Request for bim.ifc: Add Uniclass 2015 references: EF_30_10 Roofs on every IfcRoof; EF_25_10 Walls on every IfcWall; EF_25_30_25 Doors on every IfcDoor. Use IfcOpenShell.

First a look at what the model holds.

```python
import ifcopenshell

model = ifcopenshell.open("bim.ifc")
print(model.schema)
print("classifications:", [c.Name for c in model.by_type("IfcClassification")])
for ifc_class in ("IfcDoor", "IfcRoof", "IfcStair", "IfcWall", "IfcWindow"):
    print(ifc_class, len(model.by_type(ifc_class)))
```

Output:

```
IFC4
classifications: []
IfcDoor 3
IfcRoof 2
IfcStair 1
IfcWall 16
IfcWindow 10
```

```python
import ifcopenshell
import ifcopenshell.api.classification

model = ifcopenshell.open("bim.ifc")

system = ifcopenshell.api.classification.add_classification(model, classification="Uniclass 2015")

codes = {
    "IfcRoof": ("EF_30_10", "Roofs"),
    "IfcWall": ("EF_25_10", "Walls"),
    "IfcDoor": ("EF_25_30_25", "Doors"),
}
for ifc_class, (code, name) in codes.items():
    products = model.by_type(ifc_class)
    ifcopenshell.api.classification.add_reference(
        model, products=products, classification=system, identification=code, name=name
    )
    print(code, len(products))

model.write("bim_rev.ifc")
```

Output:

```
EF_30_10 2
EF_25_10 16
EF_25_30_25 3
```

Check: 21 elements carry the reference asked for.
